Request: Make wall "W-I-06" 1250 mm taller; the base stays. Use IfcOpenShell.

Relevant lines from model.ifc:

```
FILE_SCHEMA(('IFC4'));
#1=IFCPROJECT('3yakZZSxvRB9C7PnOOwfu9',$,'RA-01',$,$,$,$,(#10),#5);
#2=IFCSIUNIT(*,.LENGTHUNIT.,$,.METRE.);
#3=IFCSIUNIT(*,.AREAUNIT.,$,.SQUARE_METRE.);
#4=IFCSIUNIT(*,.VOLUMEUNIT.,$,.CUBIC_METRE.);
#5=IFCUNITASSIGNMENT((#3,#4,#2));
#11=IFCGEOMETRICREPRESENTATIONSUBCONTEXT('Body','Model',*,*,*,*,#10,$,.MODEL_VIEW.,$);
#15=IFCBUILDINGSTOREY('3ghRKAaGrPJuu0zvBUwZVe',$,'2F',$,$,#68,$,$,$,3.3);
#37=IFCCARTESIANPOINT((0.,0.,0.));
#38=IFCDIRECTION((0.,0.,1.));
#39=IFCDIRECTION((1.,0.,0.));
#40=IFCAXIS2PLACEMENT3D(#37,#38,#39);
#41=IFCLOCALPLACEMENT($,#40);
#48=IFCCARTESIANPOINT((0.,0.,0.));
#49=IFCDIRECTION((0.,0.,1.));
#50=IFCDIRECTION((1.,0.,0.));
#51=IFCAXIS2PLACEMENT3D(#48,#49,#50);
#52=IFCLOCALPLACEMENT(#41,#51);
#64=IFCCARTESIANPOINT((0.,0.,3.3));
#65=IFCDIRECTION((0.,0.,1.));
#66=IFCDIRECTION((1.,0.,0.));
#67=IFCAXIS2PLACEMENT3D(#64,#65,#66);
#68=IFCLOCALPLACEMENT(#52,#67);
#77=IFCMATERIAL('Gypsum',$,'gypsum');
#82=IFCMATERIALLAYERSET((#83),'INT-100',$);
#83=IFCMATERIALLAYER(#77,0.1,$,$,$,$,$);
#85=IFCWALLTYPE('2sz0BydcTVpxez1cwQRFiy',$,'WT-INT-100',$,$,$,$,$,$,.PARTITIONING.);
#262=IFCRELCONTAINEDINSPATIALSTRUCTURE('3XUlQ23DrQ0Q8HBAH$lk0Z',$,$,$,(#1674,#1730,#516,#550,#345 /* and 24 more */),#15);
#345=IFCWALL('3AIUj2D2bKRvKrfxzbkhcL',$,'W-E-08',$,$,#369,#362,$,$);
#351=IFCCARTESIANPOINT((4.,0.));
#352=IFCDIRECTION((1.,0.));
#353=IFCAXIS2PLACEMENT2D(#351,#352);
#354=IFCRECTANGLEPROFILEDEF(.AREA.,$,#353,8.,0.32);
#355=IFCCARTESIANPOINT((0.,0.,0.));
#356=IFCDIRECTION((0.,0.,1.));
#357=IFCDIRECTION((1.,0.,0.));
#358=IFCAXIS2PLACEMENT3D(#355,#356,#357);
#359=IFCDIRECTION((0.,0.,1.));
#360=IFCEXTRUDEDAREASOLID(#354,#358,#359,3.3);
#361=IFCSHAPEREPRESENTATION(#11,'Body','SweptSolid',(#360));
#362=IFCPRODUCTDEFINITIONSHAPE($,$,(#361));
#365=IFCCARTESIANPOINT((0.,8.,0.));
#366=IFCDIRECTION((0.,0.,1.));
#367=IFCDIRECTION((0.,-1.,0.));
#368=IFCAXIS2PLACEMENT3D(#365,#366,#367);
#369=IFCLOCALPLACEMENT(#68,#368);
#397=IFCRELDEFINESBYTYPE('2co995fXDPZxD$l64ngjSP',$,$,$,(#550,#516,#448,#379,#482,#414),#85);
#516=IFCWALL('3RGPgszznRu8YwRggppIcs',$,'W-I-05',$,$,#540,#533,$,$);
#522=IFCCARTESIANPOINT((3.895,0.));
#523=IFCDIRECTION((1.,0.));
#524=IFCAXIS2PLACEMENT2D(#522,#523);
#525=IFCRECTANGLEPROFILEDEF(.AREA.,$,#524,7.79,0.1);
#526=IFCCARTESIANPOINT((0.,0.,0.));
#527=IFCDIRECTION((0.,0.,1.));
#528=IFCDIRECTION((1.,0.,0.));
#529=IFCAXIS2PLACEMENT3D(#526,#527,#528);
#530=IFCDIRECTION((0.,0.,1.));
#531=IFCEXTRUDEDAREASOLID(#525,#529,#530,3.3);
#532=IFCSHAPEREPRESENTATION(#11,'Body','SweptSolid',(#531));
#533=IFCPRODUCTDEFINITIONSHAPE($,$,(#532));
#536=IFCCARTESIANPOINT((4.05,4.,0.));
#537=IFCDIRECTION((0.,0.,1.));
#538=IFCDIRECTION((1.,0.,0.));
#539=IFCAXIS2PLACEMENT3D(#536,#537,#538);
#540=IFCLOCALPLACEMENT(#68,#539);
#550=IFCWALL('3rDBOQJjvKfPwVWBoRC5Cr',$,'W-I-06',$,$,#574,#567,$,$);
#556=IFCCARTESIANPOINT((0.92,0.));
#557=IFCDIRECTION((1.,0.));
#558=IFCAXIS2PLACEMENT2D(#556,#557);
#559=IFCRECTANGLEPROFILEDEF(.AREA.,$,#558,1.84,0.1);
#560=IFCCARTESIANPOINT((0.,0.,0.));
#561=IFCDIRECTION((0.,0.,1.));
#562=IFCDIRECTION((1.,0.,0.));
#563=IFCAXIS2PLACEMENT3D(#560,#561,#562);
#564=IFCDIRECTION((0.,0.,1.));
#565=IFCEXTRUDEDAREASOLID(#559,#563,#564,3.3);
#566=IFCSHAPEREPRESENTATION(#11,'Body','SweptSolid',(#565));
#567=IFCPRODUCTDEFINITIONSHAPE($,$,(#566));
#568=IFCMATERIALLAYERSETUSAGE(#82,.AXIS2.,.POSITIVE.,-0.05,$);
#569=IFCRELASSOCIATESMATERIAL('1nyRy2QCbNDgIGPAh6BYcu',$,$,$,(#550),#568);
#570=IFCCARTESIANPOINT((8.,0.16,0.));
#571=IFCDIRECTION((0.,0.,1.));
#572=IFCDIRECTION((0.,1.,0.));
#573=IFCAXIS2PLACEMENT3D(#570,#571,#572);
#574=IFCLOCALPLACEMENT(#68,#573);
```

```python
import ifcopenshell
import ifcopenshell.geom
import ifcopenshell.util.representation
import ifcopenshell.util.shape

model = ifcopenshell.open("model.ifc")
settings = ifcopenshell.geom.settings()


def volume(element):
    """Net volume in cubic metres, openings subtracted."""
    shape = ifcopenshell.geom.create_shape(settings, element)
    return ifcopenshell.util.shape.get_volume(shape.geometry)


wall = model.by_guid("3rDBOQJjvKfPwVWBoRC5Cr")
before = volume(wall)

body = ifcopenshell.util.representation.get_representation(wall, "Model", "Body")
solid = body.Items[0]
old_height = solid.Depth
solid.Depth += 1.25
after = volume(wall)

print(f"height {old_height:g} -> {solid.Depth:g}, volume {before:.3f} -> {after:.3f} m3")

model.write("model_rev.ifc")
```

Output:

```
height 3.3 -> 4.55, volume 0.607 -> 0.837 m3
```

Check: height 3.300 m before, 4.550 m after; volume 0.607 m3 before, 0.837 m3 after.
